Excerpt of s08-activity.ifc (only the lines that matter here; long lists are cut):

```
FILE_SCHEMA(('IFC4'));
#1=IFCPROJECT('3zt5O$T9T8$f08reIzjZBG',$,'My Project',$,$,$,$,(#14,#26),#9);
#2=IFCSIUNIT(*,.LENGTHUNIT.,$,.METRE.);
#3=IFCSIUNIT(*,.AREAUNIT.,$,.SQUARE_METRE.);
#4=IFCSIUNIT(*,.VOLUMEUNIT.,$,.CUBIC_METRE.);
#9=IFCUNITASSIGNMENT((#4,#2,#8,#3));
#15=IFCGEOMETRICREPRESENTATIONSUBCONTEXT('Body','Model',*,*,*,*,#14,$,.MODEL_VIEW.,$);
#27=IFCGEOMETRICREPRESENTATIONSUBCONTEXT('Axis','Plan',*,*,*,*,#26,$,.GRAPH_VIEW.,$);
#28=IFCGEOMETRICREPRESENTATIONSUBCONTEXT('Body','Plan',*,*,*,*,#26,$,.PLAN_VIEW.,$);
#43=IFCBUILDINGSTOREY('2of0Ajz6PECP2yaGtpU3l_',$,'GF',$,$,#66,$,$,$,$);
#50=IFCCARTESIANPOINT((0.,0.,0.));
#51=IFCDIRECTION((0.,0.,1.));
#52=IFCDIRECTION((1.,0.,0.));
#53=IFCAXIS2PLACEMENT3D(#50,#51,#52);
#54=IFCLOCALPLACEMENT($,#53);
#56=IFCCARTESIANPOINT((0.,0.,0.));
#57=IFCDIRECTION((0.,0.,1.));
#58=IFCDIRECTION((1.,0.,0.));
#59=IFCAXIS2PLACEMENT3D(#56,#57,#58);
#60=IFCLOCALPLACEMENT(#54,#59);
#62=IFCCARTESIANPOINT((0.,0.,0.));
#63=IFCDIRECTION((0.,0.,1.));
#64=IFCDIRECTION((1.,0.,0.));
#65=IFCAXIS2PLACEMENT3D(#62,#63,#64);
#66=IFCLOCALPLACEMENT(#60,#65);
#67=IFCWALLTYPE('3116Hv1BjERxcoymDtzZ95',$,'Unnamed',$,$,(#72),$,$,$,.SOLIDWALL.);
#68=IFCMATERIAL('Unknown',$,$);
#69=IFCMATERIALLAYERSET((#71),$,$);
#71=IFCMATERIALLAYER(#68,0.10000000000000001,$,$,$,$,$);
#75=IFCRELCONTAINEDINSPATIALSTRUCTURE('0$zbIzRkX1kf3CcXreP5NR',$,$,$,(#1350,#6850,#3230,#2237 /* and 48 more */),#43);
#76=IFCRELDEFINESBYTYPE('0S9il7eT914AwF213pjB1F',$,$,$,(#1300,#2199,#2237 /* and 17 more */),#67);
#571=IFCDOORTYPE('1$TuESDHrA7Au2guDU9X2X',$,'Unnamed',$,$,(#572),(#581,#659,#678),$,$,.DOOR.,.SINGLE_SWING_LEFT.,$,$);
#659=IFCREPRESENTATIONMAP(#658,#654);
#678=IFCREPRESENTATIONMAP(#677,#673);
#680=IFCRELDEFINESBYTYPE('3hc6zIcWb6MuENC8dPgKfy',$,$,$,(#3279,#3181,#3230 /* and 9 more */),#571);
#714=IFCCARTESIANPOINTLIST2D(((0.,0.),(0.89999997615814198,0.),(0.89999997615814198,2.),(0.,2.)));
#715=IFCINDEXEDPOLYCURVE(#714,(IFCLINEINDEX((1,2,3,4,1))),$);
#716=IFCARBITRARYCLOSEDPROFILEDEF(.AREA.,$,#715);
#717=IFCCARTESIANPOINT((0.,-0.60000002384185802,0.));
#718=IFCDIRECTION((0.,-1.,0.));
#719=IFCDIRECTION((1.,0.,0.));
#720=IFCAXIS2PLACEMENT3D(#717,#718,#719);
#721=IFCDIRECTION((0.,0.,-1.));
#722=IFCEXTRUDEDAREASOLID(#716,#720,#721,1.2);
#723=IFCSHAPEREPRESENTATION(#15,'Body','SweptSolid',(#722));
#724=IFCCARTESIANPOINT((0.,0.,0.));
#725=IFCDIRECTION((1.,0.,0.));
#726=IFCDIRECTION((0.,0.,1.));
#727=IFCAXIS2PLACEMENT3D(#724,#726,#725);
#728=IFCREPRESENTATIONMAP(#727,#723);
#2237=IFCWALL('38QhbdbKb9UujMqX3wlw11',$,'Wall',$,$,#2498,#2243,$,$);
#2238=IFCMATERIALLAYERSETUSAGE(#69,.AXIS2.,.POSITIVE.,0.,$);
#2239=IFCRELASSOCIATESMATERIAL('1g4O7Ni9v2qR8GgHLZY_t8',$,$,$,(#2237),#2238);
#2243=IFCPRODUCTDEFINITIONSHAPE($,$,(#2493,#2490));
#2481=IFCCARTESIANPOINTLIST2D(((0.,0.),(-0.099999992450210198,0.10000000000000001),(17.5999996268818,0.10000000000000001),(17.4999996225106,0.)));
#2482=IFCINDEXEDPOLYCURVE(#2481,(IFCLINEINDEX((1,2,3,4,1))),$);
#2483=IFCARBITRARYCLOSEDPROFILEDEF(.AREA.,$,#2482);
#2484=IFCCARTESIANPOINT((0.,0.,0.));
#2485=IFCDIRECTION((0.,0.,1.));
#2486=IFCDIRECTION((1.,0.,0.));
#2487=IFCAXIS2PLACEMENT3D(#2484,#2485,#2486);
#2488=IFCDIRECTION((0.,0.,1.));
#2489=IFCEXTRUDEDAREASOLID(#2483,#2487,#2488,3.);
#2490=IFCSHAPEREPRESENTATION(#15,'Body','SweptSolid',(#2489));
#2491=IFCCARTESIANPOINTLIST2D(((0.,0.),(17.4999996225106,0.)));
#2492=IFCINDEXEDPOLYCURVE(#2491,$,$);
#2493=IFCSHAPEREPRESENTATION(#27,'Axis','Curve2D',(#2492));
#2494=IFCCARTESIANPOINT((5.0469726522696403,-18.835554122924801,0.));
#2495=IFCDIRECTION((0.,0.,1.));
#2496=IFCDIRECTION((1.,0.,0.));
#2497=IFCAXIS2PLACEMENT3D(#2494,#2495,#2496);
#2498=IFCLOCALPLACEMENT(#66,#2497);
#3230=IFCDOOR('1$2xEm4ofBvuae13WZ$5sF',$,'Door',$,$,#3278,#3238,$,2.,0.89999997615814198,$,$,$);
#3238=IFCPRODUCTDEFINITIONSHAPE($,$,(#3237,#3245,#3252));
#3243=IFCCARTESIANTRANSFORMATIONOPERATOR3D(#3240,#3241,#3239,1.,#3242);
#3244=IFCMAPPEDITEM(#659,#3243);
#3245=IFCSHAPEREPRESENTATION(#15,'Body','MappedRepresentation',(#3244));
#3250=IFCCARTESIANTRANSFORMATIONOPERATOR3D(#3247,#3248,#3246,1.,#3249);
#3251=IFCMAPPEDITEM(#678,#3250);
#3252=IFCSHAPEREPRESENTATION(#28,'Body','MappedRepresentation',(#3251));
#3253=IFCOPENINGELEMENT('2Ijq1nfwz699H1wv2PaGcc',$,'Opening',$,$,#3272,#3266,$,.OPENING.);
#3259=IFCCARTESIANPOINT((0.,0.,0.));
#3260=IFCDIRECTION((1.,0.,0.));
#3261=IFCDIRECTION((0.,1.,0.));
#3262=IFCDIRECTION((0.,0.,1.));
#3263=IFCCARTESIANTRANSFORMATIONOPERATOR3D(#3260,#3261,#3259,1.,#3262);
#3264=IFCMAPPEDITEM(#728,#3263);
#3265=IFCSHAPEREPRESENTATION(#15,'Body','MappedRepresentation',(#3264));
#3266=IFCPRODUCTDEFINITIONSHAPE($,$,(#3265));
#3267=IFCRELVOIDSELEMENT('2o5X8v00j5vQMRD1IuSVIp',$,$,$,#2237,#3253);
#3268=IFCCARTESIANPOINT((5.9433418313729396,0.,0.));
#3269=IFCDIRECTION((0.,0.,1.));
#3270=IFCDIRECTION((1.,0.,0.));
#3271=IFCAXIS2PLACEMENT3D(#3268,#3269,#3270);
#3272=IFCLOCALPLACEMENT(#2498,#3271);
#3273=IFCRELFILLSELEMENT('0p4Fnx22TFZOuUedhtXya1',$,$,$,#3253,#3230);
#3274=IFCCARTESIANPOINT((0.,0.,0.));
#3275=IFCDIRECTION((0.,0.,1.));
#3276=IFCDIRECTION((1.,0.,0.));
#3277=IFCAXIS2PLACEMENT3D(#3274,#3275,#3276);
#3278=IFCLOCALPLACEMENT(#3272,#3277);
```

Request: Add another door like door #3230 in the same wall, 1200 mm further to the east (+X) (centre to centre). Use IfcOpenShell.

```python
import ifcopenshell
import ifcopenshell.api.feature
import ifcopenshell.api.geometry
import ifcopenshell.api.root
import ifcopenshell.geom
import ifcopenshell.util.element
import ifcopenshell.util.placement
import ifcopenshell.util.shape

model = ifcopenshell.open("s08-activity.ifc")
settings = ifcopenshell.geom.settings()


def volume(element):
    """Net volume in cubic metres, openings subtracted."""
    shape = ifcopenshell.geom.create_shape(settings, element)
    return ifcopenshell.util.shape.get_volume(shape.geometry)


door = model.by_guid("1$2xEm4ofBvuae13WZ$5sF")
opening = door.FillsVoids[0].RelatingOpeningElement
wall = opening.VoidsElements[0].RelatingBuildingElement
before = volume(wall)
shift = ifcopenshell.util.placement.get_local_placement(wall.ObjectPlacement)[:3, 0] * 1.2

# copy_class copies the void relationship, type, container and properties, but no geometry.
new_opening = ifcopenshell.api.root.copy_class(model, product=opening)
new_opening.Representation = ifcopenshell.util.element.copy_deep(
    model, opening.Representation, exclude=["IfcGeometricRepresentationContext", "IfcRepresentationMap"]
)
new_door = ifcopenshell.api.root.copy_class(model, product=door)
new_door.Representation = ifcopenshell.util.element.copy_deep(
    model, door.Representation, exclude=["IfcGeometricRepresentationContext", "IfcRepresentationMap"]
)
ifcopenshell.api.feature.add_filling(model, opening=new_opening, element=new_door)

for old, new in ((opening, new_opening), (door, new_door)):
    matrix = ifcopenshell.util.placement.get_local_placement(old.ObjectPlacement)
    matrix[:3, 3] += shift
    ifcopenshell.api.geometry.edit_object_placement(model, product=new, matrix=matrix, is_si=False)

after = volume(wall)

print(f"wall volume {before:.3f} -> {after:.3f} m3")

model.write("s08-activity-out.ifc")
```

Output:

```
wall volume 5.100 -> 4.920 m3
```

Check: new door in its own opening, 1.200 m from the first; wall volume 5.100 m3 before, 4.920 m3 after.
